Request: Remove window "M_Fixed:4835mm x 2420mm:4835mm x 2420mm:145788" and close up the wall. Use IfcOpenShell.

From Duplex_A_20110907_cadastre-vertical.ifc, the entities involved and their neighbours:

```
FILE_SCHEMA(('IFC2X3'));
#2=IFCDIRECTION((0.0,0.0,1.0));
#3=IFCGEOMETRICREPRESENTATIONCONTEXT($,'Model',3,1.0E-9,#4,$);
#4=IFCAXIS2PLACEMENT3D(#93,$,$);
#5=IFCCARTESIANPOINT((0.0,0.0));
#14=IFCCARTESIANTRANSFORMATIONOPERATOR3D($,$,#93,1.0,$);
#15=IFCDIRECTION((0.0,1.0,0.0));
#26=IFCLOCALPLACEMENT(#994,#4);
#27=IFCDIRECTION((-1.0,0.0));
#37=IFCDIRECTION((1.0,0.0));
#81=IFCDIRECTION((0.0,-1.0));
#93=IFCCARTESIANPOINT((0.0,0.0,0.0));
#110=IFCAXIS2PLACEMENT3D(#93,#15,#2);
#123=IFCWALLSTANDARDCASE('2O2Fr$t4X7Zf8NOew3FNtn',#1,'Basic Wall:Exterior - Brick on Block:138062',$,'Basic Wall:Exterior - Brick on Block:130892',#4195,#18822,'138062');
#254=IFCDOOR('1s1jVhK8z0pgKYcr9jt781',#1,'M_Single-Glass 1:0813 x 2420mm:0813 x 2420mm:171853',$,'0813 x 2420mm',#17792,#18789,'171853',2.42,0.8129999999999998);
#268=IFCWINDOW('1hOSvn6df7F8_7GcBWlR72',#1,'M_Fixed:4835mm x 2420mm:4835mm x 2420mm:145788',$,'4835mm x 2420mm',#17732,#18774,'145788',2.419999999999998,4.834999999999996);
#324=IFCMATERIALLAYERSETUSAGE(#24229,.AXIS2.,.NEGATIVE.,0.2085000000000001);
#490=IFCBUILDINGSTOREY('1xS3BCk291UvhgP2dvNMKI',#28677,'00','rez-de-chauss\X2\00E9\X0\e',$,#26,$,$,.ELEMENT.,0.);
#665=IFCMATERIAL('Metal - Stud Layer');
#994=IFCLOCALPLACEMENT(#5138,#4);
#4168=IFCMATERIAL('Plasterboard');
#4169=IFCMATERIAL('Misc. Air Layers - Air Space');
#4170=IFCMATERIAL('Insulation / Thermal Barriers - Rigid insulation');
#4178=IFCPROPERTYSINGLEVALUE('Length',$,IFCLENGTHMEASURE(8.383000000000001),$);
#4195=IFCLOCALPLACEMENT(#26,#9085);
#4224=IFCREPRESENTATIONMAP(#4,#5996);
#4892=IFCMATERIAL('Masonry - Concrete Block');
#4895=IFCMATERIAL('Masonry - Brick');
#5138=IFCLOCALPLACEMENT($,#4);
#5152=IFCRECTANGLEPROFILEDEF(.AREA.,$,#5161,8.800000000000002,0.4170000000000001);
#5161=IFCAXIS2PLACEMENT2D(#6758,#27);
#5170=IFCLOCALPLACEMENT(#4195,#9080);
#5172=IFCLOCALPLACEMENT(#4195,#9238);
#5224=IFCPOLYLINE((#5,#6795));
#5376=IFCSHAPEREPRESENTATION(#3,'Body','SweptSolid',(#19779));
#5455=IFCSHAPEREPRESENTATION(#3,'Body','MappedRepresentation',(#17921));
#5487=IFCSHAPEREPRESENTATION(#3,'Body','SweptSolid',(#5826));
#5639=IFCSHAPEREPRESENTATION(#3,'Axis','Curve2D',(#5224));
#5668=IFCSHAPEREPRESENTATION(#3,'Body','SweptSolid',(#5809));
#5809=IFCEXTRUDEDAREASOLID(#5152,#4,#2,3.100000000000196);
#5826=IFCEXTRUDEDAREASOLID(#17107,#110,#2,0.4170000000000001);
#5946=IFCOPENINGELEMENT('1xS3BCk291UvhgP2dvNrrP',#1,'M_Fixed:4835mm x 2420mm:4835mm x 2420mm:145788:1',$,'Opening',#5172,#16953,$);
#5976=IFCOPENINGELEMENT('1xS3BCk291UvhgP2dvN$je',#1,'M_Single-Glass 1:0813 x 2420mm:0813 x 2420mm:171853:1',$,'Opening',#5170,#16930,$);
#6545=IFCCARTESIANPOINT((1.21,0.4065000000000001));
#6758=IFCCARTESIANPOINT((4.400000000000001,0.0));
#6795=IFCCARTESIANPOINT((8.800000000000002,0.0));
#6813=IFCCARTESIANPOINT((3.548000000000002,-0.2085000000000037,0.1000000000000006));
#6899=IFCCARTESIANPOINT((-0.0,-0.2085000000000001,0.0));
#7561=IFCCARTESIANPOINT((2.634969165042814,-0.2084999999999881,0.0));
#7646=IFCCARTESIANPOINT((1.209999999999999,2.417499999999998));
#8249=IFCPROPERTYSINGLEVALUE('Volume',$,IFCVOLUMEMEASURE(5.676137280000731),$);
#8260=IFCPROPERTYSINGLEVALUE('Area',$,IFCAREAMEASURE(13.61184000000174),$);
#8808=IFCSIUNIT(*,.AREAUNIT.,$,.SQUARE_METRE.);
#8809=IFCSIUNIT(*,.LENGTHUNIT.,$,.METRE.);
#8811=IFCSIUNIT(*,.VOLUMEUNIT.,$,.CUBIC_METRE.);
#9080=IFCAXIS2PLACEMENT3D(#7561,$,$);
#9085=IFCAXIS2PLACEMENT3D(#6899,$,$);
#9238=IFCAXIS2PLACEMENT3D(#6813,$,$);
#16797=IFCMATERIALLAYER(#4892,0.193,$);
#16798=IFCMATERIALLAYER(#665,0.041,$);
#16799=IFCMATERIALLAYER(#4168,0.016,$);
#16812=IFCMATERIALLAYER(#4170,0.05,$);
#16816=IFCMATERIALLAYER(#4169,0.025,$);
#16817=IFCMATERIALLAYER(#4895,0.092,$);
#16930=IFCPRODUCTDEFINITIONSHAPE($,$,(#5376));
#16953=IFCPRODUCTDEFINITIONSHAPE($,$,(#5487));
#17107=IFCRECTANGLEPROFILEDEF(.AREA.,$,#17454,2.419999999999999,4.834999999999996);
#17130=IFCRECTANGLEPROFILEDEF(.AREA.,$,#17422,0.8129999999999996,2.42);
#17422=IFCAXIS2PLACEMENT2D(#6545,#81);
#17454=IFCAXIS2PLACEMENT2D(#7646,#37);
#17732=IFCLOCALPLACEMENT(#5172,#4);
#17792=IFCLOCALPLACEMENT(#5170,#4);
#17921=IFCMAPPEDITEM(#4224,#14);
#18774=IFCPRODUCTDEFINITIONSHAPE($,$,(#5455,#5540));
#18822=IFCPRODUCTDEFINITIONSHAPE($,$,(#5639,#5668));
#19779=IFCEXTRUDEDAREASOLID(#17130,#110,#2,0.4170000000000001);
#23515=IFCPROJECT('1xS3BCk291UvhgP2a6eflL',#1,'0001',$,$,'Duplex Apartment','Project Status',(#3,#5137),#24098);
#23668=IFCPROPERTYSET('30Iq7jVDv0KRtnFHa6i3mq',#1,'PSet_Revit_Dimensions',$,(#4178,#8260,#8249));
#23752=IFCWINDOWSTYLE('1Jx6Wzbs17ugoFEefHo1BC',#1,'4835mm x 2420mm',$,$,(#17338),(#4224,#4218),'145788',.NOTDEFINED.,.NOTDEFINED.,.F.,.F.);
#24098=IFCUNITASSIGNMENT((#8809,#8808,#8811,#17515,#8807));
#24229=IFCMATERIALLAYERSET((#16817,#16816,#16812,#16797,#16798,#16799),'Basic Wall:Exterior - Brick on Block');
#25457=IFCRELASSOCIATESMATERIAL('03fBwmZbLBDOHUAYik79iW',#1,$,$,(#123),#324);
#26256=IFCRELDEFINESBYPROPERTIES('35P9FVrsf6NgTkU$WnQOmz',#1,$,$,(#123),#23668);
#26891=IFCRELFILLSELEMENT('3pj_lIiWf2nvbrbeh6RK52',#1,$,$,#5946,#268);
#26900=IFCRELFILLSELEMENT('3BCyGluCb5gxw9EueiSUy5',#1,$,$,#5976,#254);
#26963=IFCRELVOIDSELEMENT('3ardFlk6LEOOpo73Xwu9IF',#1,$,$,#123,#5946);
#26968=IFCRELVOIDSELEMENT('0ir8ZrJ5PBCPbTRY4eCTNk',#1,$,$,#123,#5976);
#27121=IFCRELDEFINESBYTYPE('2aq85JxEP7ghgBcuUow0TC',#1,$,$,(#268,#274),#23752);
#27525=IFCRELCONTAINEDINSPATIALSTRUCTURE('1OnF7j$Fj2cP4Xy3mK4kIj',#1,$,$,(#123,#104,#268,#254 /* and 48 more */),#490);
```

```python
import ifcopenshell
import ifcopenshell.api.feature
import ifcopenshell.api.pset
import ifcopenshell.api.root
import ifcopenshell.geom
import ifcopenshell.util.element
import ifcopenshell.util.shape
import ifcopenshell.util.unit

model = ifcopenshell.open("Duplex_A_20110907_cadastre-vertical.ifc")
area_scale = ifcopenshell.util.unit.calculate_unit_scale(model, "AREAUNIT")
volume_scale = ifcopenshell.util.unit.calculate_unit_scale(model, "VOLUMEUNIT")
settings = ifcopenshell.geom.settings()


def volume(element):
    """Net volume in cubic metres, openings subtracted."""
    shape = ifcopenshell.geom.create_shape(settings, element)
    return ifcopenshell.util.shape.get_volume(shape.geometry)


window = model.by_id(268)
opening = window.FillsVoids[0].RelatingOpeningElement
wall = opening.VoidsElements[0].RelatingBuildingElement
before = volume(wall)

ifcopenshell.api.root.remove_product(model, product=window)
ifcopenshell.api.feature.remove_feature(model, feature=opening)

after = volume(wall)
thickness = 0.417  # wall thickness in metres

# Update the wall's stored quantities.
pset = model.by_id(ifcopenshell.util.element.get_pset(wall, "PSet_Revit_Dimensions", should_inherit=False)["id"])
ifcopenshell.api.pset.edit_pset(model, pset=pset, properties={
    "Area": model.create_entity("IfcAreaMeasure", after / thickness / area_scale),
    "Volume": model.create_entity("IfcVolumeMeasure", after / volume_scale),
})

print(f"wall volume {before:.3f} -> {after:.3f} m3")

model.write("Duplex_A_20110907_cadastre-vertical_rev.ifc")
```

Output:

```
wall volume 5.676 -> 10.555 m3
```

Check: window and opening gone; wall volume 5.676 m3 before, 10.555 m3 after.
